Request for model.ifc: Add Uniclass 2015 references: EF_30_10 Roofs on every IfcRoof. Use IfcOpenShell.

First a look at what the model holds.

```python
import ifcopenshell

model = ifcopenshell.open("model.ifc")
print(model.schema)
print("classifications:", [c.Name for c in model.by_type("IfcClassification")])
for ifc_class in ("IfcDoor", "IfcRoof", "IfcStair", "IfcWall", "IfcWindow"):
    print(ifc_class, len(model.by_type(ifc_class)))
```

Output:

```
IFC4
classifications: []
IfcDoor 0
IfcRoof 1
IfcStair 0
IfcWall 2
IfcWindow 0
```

```python
import ifcopenshell
import ifcopenshell.api.classification

model = ifcopenshell.open("model.ifc")

system = ifcopenshell.api.classification.add_classification(model, classification="Uniclass 2015")

codes = {
    "IfcRoof": ("EF_30_10", "Roofs"),
}
for ifc_class, (code, name) in codes.items():
    products = model.by_type(ifc_class)
    ifcopenshell.api.classification.add_reference(
        model, products=products, classification=system, identification=code, name=name
    )
    print(code, len(products))

model.write("model_updated.ifc")
```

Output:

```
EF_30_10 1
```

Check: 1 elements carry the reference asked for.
